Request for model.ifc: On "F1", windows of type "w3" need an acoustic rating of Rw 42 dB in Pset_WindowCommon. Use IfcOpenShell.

First a look at what the model holds.

```python
import ifcopenshell
import ifcopenshell.util.element

model = ifcopenshell.open("model.ifc")
print(model.schema)
storey = next(s for s in model.by_type("IfcBuildingStorey") if s.Name == "F1")
windows = [e for e in ifcopenshell.util.element.get_decomposition(storey) if e.is_a("IfcWindow")]
seen = {}
for e in windows:
    element_type = ifcopenshell.util.element.get_type(e)
    key = (element_type.Name if element_type != e and element_type else None, ifcopenshell.util.element.get_pset(e, "Pset_WindowCommon", "AcousticRating"))
    seen[key] = seen.get(key, 0) + 1
for (name, value), count in sorted(seen.items(), key=str):
    print(count, "x", name, "|", value)
```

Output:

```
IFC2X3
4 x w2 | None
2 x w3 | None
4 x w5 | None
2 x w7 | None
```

```python
import ifcopenshell
import ifcopenshell.api.pset
import ifcopenshell.util.element

model = ifcopenshell.open("model.ifc")

storey = next(s for s in model.by_type("IfcBuildingStorey") if s.Name == "F1")
windows = [e for e in ifcopenshell.util.element.get_decomposition(storey) if e.is_a("IfcWindow")]

count = 0
for e in windows:
    element_type = ifcopenshell.util.element.get_type(e)
    if element_type in (None, e) or element_type.Name != "w3":
        continue
    # add_pset returns the element's existing set when there is one.
    pset = ifcopenshell.api.pset.add_pset(model, product=e, name="Pset_WindowCommon")
    ifcopenshell.api.pset.edit_pset(model, pset=pset, properties={"AcousticRating": "Rw 42 dB"})
    count += 1

print(count, "windows updated")

model.write("model_rev.ifc")
```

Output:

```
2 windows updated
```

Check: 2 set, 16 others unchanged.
